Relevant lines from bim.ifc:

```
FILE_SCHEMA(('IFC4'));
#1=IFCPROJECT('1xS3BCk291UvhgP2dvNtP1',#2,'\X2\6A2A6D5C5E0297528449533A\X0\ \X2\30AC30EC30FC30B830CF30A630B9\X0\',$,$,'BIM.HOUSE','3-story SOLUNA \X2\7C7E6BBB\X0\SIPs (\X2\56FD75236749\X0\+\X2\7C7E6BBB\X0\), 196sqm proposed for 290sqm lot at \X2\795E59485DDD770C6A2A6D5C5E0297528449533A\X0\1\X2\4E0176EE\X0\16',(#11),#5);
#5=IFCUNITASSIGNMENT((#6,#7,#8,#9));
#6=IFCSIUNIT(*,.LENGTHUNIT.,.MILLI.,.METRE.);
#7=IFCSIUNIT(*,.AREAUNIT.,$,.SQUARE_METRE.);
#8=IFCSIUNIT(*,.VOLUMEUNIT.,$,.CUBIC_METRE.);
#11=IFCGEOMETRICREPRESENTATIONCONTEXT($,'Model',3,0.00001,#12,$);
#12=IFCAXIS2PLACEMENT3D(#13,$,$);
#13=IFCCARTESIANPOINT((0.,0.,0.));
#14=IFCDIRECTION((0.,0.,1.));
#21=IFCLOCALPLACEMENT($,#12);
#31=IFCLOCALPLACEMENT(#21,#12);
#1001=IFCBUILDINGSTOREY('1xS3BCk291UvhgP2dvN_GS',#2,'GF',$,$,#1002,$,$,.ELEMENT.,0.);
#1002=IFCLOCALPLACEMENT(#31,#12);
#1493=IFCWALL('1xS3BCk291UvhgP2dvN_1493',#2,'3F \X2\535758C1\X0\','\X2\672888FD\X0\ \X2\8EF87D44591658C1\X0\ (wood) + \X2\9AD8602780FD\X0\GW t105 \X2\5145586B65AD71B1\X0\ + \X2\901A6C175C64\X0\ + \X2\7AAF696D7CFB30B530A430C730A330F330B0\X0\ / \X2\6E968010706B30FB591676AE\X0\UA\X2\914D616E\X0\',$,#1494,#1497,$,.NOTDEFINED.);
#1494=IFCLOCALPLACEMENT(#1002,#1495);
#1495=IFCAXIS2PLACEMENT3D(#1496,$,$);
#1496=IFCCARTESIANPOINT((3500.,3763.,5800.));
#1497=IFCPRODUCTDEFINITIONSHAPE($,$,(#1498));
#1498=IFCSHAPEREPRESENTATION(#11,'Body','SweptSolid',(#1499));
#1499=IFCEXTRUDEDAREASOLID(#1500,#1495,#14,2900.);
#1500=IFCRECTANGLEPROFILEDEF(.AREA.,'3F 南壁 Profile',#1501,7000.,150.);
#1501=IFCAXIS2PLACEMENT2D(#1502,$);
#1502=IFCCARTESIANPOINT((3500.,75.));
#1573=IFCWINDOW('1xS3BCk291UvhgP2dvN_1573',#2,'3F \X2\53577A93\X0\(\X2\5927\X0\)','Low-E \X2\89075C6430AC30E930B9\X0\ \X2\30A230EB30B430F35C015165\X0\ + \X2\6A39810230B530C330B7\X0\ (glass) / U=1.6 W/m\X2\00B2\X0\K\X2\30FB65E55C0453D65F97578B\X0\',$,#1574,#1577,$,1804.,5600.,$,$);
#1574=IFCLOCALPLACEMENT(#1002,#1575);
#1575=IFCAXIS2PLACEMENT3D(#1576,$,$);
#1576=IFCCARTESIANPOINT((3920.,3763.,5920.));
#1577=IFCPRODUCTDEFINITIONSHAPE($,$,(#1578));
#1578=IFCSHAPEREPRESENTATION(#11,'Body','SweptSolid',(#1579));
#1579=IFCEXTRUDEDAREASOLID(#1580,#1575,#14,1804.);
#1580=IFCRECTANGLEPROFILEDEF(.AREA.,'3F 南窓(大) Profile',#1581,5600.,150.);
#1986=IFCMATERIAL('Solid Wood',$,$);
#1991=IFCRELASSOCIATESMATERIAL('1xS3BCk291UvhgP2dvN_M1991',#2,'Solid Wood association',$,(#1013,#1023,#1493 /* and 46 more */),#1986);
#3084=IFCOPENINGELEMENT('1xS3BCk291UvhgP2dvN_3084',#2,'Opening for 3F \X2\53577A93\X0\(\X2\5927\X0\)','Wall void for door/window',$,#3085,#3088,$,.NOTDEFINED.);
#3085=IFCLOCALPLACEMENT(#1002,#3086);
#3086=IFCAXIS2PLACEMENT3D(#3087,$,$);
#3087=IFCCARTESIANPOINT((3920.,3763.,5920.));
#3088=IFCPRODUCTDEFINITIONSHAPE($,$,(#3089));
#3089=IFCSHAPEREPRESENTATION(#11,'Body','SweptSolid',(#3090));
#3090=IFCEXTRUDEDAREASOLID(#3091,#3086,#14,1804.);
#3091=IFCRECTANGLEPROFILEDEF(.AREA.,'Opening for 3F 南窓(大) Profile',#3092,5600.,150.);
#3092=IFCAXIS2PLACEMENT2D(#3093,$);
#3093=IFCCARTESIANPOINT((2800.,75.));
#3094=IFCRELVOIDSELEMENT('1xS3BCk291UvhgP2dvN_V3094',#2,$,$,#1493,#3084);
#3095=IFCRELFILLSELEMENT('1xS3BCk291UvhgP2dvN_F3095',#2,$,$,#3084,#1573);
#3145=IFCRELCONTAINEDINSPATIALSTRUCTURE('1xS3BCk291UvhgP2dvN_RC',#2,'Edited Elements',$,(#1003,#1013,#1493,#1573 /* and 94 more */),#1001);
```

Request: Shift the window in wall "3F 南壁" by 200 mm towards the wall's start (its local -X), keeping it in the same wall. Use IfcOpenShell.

```python
import ifcopenshell
import ifcopenshell.api.geometry
import ifcopenshell.util.placement

model = ifcopenshell.open("bim.ifc")

window = model.by_guid("1xS3BCk291UvhgP2dvN_1573")
opening = window.FillsVoids[0].RelatingOpeningElement
wall = opening.VoidsElements[0].RelatingBuildingElement

wall_matrix = ifcopenshell.util.placement.get_local_placement(wall.ObjectPlacement)
shift = wall_matrix[:3, 0] * -200.0
before = ifcopenshell.util.placement.get_local_placement(window.ObjectPlacement)[:3, 3].copy()

# The window is not placed relative to its opening, so move both.
for product in (opening, window):
    matrix = ifcopenshell.util.placement.get_local_placement(product.ObjectPlacement)
    matrix[:3, 3] += shift
    ifcopenshell.api.geometry.edit_object_placement(model, product=product, matrix=matrix, is_si=False)

after = ifcopenshell.util.placement.get_local_placement(window.ObjectPlacement)[:3, 3]
print("window moved by", (after - before).round(3) + 0.0)

model.write("bim_rev.ifc")
```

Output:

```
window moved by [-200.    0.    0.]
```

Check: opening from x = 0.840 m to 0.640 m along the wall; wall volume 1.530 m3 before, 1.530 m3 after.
